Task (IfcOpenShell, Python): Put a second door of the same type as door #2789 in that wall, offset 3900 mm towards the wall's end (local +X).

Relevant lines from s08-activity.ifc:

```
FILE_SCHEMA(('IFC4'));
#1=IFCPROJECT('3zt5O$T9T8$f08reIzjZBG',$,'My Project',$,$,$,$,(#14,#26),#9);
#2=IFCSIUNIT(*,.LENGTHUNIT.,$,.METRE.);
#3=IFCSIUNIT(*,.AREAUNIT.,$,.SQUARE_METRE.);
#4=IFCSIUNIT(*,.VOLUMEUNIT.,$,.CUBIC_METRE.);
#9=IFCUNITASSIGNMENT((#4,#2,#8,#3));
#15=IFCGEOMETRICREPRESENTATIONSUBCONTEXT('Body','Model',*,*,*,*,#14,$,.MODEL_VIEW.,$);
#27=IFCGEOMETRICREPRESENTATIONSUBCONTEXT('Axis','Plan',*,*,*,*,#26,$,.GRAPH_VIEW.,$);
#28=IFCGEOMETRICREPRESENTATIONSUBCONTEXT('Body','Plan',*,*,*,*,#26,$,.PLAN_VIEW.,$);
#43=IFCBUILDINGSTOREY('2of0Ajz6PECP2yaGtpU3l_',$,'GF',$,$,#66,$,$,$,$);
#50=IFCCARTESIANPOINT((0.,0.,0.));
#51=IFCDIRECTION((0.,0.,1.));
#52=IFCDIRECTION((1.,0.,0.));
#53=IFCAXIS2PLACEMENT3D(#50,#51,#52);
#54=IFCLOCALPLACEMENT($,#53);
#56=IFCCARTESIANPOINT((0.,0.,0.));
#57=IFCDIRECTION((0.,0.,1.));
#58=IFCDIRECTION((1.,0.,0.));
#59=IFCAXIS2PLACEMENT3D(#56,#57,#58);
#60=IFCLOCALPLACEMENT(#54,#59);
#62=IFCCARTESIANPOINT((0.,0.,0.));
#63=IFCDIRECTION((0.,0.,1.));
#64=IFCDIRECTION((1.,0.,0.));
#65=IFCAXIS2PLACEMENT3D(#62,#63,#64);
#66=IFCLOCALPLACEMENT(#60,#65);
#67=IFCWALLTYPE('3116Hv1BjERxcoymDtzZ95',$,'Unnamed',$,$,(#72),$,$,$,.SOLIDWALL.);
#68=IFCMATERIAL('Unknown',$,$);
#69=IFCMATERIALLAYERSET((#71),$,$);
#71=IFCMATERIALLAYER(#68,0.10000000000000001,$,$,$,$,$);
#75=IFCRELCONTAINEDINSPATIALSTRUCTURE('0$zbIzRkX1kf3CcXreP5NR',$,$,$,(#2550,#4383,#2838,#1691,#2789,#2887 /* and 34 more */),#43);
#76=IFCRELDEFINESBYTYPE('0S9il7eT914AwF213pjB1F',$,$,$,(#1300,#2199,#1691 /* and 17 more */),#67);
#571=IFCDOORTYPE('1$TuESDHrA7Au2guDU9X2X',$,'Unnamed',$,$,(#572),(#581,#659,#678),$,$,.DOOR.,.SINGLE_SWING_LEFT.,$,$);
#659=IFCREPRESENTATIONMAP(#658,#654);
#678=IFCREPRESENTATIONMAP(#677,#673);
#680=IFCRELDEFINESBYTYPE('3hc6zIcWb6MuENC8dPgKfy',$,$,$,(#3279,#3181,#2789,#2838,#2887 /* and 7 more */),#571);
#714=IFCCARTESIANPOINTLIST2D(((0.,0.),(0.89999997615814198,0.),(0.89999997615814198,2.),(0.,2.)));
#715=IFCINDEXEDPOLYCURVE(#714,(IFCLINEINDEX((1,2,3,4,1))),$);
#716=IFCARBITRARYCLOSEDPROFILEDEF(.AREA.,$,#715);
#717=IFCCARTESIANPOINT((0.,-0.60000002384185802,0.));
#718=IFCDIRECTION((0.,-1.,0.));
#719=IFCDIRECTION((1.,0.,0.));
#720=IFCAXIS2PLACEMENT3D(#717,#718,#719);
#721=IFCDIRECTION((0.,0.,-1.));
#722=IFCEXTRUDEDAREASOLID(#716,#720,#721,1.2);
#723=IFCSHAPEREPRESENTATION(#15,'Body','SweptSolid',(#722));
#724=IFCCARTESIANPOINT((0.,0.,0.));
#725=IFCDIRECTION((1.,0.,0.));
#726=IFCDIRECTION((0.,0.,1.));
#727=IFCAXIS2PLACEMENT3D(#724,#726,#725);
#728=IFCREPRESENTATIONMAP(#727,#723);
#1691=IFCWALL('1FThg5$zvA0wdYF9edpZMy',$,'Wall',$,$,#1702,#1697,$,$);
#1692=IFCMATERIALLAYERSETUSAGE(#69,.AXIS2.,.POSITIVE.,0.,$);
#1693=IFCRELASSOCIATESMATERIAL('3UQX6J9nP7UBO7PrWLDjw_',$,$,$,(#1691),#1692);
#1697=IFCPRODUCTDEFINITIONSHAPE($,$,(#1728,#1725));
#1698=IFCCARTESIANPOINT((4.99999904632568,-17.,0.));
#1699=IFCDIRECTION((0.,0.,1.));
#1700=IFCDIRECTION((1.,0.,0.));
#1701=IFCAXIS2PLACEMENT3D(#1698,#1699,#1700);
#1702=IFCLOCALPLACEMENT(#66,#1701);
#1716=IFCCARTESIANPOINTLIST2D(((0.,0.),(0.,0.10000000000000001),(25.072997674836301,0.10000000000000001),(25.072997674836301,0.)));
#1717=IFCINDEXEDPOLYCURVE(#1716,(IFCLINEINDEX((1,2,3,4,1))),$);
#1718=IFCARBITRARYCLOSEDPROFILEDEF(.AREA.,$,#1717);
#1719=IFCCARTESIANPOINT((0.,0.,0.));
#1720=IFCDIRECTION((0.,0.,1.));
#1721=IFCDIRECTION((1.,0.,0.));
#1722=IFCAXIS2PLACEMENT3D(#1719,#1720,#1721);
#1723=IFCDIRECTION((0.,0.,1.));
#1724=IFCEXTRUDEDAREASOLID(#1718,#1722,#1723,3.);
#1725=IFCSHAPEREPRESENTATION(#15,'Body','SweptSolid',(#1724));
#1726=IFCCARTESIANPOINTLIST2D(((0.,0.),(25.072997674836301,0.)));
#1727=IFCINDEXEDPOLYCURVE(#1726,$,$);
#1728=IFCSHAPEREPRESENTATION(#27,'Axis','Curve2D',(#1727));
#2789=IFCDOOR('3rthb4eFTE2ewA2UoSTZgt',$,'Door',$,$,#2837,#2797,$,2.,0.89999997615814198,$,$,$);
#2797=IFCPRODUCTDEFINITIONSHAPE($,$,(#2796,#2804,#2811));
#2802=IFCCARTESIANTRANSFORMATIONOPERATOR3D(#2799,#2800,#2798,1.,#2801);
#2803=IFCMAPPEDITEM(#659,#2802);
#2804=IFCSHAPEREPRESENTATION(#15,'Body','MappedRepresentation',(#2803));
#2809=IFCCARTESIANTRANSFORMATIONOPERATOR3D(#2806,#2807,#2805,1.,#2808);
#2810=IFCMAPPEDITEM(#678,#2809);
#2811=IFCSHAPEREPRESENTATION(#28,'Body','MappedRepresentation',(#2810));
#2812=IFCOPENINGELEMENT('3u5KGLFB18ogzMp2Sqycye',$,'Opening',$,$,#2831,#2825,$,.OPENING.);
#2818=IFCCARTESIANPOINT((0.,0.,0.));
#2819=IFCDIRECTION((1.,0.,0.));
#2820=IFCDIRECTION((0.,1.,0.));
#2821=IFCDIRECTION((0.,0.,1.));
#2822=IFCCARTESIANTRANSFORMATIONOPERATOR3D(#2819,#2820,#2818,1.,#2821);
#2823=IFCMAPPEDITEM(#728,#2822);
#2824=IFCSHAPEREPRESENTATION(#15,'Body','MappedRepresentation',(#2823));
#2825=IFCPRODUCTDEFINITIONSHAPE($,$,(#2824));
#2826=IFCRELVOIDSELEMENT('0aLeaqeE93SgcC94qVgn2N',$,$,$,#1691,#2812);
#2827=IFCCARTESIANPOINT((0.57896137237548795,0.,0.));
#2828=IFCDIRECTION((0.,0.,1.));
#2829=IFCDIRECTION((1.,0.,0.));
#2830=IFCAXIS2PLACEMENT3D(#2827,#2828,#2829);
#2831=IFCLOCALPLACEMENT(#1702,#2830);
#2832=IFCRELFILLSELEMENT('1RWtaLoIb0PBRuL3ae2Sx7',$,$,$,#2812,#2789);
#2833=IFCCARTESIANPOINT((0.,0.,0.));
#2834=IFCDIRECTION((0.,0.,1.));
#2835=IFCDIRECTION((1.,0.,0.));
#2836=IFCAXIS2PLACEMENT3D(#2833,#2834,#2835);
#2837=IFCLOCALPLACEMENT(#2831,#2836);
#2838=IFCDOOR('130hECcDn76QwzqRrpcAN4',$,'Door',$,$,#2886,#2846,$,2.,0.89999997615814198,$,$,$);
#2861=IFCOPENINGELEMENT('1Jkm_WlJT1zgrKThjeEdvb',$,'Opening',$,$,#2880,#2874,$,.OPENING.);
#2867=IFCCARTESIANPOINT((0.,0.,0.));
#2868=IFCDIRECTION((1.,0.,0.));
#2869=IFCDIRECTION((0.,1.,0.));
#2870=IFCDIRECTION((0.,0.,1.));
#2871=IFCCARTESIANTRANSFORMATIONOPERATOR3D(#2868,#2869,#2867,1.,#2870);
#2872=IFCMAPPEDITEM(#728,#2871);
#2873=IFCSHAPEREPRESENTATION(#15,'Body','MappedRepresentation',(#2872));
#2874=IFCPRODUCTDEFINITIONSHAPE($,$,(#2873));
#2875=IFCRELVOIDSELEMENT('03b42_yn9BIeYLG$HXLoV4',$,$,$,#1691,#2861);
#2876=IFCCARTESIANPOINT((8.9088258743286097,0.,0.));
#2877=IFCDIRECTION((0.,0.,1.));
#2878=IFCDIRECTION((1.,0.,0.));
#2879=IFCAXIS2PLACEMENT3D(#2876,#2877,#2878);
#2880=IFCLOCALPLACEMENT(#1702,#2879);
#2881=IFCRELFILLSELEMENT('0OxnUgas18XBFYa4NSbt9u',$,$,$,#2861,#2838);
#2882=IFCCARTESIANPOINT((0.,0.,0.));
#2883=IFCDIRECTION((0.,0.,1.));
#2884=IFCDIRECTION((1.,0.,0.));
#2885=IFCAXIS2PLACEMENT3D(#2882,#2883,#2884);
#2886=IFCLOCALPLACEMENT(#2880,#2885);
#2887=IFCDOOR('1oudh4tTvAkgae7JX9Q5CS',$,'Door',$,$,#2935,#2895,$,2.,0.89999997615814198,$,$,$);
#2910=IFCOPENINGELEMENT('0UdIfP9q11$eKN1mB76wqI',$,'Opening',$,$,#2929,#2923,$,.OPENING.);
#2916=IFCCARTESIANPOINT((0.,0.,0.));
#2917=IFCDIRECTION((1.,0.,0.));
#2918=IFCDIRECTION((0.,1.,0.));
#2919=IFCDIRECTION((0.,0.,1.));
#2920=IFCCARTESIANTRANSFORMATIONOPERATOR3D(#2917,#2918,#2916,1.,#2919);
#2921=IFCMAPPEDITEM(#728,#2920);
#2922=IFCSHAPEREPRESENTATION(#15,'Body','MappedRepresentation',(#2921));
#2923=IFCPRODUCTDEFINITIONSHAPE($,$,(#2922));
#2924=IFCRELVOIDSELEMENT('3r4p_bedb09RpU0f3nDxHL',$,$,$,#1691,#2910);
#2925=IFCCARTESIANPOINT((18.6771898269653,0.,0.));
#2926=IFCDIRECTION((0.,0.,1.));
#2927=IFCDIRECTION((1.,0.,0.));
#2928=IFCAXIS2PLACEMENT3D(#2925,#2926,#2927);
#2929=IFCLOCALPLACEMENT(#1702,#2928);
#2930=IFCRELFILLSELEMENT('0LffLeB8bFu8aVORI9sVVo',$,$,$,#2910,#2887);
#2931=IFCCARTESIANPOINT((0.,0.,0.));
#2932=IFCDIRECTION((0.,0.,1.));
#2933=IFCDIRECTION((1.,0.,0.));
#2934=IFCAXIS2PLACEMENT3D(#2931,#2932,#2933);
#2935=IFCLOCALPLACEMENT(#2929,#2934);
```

```python
import ifcopenshell
import ifcopenshell.api.feature
import ifcopenshell.api.geometry
import ifcopenshell.api.root
import ifcopenshell.geom
import ifcopenshell.util.element
import ifcopenshell.util.placement
import ifcopenshell.util.shape
import ifcopenshell.util.unit

model = ifcopenshell.open("s08-activity.ifc")
unit_scale = ifcopenshell.util.unit.calculate_unit_scale(model)
settings = ifcopenshell.geom.settings()


def volume(element):
    """Net volume in cubic metres, openings subtracted."""
    shape = ifcopenshell.geom.create_shape(settings, element)
    return ifcopenshell.util.shape.get_volume(shape.geometry)


door = model.by_guid("3rthb4eFTE2ewA2UoSTZgt")
opening = door.FillsVoids[0].RelatingOpeningElement
wall = opening.VoidsElements[0].RelatingBuildingElement
before = volume(wall)
shift = ifcopenshell.util.placement.get_local_placement(wall.ObjectPlacement)[:3, 0] * 3.9 / unit_scale

# copy_class copies the void relationship, type, container and properties, but no geometry.
new_opening = ifcopenshell.api.root.copy_class(model, product=opening)
new_opening.Representation = ifcopenshell.util.element.copy_deep(
    model, opening.Representation, exclude=["IfcGeometricRepresentationContext", "IfcRepresentationMap"]
)
new_door = ifcopenshell.api.root.copy_class(model, product=door)
new_door.Representation = ifcopenshell.util.element.copy_deep(
    model, door.Representation, exclude=["IfcGeometricRepresentationContext", "IfcRepresentationMap"]
)
ifcopenshell.api.feature.add_filling(model, opening=new_opening, element=new_door)

for old, new in ((opening, new_opening), (door, new_door)):
    matrix = ifcopenshell.util.placement.get_local_placement(old.ObjectPlacement)
    matrix[:3, 3] += shift
    ifcopenshell.api.geometry.edit_object_placement(model, product=new, matrix=matrix, is_si=False)

after = volume(wall)

print(f"wall volume {before:.3f} -> {after:.3f} m3")

model.write("s08-activity_edited.ifc")
```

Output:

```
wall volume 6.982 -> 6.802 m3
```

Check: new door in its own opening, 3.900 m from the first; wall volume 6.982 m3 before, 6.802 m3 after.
